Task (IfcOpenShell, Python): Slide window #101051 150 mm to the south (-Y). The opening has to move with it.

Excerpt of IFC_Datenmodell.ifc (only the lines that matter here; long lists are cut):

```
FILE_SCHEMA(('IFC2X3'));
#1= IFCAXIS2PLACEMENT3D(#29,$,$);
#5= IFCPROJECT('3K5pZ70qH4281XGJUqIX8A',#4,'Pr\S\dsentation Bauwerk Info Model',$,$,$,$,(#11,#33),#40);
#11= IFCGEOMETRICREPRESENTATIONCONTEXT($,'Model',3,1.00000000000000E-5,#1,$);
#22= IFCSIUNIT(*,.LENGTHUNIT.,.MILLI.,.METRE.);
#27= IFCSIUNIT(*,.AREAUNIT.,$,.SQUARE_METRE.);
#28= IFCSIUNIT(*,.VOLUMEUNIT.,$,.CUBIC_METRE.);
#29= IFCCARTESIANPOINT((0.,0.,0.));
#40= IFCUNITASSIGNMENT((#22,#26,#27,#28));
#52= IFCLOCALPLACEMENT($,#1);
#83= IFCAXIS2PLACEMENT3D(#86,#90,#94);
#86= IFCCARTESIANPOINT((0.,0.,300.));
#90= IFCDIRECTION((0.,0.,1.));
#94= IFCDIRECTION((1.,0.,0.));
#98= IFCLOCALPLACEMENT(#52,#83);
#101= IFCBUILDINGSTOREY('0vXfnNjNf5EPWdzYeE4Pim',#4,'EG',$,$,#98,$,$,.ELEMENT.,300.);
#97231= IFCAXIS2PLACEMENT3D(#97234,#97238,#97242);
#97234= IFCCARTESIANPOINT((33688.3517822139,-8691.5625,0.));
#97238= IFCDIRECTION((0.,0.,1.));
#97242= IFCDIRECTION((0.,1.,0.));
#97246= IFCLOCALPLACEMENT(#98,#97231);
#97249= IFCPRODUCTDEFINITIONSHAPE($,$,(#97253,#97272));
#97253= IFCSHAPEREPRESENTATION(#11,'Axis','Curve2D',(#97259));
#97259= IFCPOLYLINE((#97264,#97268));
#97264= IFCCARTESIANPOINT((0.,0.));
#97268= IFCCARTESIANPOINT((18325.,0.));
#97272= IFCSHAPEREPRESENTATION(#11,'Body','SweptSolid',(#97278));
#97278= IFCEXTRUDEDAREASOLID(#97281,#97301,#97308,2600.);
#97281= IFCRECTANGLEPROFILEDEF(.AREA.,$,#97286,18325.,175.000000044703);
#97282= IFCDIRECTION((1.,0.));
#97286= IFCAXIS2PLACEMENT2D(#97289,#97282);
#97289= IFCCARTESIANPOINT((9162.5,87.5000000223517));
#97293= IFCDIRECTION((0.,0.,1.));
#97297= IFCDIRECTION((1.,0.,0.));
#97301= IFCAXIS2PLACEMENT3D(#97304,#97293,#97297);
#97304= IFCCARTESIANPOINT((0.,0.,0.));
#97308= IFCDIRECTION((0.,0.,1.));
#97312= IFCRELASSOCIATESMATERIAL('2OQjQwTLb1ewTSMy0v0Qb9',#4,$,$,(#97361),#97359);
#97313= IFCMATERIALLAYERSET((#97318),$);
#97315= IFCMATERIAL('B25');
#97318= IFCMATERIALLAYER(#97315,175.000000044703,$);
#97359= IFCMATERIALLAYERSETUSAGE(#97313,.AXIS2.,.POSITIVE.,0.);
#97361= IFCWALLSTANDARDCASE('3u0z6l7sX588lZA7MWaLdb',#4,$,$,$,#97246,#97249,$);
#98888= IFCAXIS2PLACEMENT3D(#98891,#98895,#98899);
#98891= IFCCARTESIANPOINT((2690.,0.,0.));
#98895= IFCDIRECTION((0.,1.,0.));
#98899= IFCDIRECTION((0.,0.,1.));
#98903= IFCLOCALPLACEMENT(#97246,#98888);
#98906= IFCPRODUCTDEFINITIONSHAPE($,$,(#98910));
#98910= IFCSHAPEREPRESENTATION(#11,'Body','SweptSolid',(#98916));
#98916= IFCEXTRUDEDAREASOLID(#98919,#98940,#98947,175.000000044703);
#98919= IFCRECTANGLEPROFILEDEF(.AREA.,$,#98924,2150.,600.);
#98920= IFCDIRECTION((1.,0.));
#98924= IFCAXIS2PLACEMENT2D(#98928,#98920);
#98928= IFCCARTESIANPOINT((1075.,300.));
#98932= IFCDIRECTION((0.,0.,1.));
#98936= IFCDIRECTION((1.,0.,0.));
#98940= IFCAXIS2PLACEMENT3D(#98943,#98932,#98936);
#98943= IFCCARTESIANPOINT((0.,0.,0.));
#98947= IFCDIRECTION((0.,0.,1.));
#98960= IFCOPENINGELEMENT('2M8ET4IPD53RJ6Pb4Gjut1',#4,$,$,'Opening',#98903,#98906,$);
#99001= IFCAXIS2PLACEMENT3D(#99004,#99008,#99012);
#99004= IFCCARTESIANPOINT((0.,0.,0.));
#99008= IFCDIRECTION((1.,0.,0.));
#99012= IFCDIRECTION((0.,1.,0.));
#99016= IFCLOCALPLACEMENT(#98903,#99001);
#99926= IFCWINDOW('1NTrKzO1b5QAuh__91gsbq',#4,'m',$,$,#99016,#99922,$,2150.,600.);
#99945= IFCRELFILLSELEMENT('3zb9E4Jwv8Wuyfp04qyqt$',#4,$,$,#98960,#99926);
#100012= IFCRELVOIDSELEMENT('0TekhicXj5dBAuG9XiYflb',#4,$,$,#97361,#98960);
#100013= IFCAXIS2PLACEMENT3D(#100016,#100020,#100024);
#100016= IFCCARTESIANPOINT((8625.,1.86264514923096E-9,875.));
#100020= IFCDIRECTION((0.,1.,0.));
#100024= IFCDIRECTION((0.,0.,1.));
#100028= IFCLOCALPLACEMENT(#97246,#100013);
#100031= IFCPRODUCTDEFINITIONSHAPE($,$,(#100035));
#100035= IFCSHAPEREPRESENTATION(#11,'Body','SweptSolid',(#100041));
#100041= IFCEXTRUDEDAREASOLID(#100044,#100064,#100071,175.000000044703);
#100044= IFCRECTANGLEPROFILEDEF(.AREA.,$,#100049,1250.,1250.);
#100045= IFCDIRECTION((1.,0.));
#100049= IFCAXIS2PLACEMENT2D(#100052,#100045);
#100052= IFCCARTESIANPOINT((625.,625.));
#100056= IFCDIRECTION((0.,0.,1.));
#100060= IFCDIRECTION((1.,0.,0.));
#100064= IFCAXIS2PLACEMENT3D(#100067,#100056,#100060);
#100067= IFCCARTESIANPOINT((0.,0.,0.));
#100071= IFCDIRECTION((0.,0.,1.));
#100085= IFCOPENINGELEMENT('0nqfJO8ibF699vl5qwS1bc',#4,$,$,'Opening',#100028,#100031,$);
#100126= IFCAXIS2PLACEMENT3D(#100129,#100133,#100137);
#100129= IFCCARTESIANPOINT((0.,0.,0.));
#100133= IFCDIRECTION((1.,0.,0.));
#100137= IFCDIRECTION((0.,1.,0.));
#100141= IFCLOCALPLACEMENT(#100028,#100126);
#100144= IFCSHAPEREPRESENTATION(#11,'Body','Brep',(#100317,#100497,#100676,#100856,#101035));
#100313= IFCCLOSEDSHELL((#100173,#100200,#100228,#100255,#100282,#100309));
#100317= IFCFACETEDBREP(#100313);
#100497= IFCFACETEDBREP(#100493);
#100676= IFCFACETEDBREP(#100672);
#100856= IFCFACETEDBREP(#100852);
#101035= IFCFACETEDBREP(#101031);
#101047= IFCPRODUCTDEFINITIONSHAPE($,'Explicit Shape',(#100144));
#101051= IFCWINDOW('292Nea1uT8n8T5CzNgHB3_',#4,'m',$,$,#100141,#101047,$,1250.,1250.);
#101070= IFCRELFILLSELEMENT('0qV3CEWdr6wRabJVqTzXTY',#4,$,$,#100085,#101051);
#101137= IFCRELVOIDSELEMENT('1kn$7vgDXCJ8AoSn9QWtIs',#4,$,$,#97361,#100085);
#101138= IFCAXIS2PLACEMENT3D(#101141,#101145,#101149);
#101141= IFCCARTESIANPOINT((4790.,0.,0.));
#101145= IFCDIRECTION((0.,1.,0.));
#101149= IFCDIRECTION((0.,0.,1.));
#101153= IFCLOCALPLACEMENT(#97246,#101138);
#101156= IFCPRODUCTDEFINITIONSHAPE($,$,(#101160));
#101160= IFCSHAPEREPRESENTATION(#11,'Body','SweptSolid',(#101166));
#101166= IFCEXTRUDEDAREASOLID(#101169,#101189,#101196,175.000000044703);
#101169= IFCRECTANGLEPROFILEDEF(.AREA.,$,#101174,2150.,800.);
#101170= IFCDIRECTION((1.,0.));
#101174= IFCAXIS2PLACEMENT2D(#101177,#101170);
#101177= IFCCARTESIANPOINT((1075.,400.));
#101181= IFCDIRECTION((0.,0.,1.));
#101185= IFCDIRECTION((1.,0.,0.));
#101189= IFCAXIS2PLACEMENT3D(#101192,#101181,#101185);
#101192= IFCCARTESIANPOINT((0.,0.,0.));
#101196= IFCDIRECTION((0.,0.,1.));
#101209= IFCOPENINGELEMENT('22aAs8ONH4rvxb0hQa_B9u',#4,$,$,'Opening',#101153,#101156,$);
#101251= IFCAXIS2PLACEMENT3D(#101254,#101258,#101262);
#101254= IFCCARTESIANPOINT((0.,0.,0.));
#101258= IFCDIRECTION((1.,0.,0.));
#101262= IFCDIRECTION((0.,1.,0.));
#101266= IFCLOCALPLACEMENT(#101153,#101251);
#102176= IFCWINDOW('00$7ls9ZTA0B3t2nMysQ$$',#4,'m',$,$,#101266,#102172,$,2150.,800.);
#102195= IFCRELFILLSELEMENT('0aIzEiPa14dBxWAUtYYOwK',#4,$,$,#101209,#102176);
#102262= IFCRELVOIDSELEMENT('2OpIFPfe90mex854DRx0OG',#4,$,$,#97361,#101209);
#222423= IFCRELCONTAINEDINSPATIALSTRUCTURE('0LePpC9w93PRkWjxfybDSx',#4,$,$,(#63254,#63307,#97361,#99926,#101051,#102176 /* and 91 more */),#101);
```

```python
import ifcopenshell
import ifcopenshell.api.geometry
import ifcopenshell.util.placement
import ifcopenshell.util.unit

model = ifcopenshell.open("IFC_Datenmodell.ifc")
unit_scale = ifcopenshell.util.unit.calculate_unit_scale(model)

window = model.by_guid("292Nea1uT8n8T5CzNgHB3_")
opening = window.FillsVoids[0].RelatingOpeningElement
wall = opening.VoidsElements[0].RelatingBuildingElement

wall_matrix = ifcopenshell.util.placement.get_local_placement(wall.ObjectPlacement)
shift = wall_matrix[:3, 0] * -0.15 / unit_scale
before = ifcopenshell.util.placement.get_local_placement(window.ObjectPlacement)[:3, 3].copy()

# The window is placed relative to its opening, so it follows when the opening moves.
matrix = ifcopenshell.util.placement.get_local_placement(opening.ObjectPlacement)
matrix[:3, 3] += shift
ifcopenshell.api.geometry.edit_object_placement(
    model, product=opening, matrix=matrix, is_si=False, should_transform_children=True
)

after = ifcopenshell.util.placement.get_local_placement(window.ObjectPlacement)[:3, 3]
print("window moved by", (after - before).round(3) + 0.0)

model.write("IFC_Datenmodell_v2.ifc")
```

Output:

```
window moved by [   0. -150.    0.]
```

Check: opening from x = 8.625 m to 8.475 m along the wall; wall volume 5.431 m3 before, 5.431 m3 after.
